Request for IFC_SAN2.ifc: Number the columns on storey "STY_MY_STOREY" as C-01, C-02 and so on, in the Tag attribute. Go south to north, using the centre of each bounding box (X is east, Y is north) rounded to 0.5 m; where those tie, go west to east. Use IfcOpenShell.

First a look at what the model holds.

```python
import ifcopenshell
import ifcopenshell.util.element
import ifcopenshell.util.placement

model = ifcopenshell.open("IFC_SAN2.ifc")
print(model.schema)
storey = next(s for s in model.by_type("IfcBuildingStorey") if s.Name == "STY_MY_STOREY")
columns = [e for e in ifcopenshell.util.element.get_decomposition(storey) if e.is_a("IfcColumn")]
for e in sorted(columns, key=lambda e: e.id()):
    origin = ifcopenshell.util.placement.get_local_placement(e.ObjectPlacement)[:3, 3]
    print(e.id(), e.Tag, e.Name, origin.round(2) + 0.0, sep=" | ")
```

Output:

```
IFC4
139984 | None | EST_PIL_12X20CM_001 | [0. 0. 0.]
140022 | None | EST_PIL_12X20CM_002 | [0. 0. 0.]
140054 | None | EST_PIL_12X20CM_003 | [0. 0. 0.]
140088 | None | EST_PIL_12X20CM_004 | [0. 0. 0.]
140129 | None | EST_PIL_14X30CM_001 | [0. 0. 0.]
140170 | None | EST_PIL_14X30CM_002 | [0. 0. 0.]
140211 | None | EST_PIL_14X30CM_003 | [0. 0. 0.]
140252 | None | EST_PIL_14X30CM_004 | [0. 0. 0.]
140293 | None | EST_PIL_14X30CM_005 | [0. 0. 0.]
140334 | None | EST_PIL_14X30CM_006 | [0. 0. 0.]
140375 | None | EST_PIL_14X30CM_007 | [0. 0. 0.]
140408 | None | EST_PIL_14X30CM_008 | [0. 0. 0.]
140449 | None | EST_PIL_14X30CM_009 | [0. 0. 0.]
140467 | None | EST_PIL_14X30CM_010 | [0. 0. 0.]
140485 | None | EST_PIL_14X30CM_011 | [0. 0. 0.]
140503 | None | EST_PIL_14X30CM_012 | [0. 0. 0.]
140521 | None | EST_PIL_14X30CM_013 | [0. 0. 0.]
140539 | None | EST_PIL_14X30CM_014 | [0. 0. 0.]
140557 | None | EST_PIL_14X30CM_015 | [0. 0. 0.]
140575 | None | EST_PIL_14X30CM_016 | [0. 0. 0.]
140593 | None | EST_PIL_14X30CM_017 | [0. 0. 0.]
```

```python
import ifcopenshell
import ifcopenshell.geom
import ifcopenshell.util.element
import ifcopenshell.util.shape

model = ifcopenshell.open("IFC_SAN2.ifc")
settings = ifcopenshell.geom.settings()
settings.set("use-world-coords", True)


def centre(element):
    shape = ifcopenshell.geom.create_shape(settings, element)
    return ifcopenshell.util.shape.get_bbox_centroid(shape.geometry)


storey = next(s for s in model.by_type("IfcBuildingStorey") if s.Name == "STY_MY_STOREY")
columns = [e for e in ifcopenshell.util.element.get_decomposition(storey) if e.is_a("IfcColumn")]

# Insertion points can sit at a corner or the storey origin, so sort by the geometry (in metres).
centres = {e: centre(e) for e in columns}
columns.sort(key=lambda e: (round(centres[e][1] / 0.5), centres[e][0]))

for i, e in enumerate(columns, start=1):
    number = f"C-{i:02d}"
    e.Tag = number
    print(e.id(), number)

model.write("IFC_SAN2-out.ifc")
```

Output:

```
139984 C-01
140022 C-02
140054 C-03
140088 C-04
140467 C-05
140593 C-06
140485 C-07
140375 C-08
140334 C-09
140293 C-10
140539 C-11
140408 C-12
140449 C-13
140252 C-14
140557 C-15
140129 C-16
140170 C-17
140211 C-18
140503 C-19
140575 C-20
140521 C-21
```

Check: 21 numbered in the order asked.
